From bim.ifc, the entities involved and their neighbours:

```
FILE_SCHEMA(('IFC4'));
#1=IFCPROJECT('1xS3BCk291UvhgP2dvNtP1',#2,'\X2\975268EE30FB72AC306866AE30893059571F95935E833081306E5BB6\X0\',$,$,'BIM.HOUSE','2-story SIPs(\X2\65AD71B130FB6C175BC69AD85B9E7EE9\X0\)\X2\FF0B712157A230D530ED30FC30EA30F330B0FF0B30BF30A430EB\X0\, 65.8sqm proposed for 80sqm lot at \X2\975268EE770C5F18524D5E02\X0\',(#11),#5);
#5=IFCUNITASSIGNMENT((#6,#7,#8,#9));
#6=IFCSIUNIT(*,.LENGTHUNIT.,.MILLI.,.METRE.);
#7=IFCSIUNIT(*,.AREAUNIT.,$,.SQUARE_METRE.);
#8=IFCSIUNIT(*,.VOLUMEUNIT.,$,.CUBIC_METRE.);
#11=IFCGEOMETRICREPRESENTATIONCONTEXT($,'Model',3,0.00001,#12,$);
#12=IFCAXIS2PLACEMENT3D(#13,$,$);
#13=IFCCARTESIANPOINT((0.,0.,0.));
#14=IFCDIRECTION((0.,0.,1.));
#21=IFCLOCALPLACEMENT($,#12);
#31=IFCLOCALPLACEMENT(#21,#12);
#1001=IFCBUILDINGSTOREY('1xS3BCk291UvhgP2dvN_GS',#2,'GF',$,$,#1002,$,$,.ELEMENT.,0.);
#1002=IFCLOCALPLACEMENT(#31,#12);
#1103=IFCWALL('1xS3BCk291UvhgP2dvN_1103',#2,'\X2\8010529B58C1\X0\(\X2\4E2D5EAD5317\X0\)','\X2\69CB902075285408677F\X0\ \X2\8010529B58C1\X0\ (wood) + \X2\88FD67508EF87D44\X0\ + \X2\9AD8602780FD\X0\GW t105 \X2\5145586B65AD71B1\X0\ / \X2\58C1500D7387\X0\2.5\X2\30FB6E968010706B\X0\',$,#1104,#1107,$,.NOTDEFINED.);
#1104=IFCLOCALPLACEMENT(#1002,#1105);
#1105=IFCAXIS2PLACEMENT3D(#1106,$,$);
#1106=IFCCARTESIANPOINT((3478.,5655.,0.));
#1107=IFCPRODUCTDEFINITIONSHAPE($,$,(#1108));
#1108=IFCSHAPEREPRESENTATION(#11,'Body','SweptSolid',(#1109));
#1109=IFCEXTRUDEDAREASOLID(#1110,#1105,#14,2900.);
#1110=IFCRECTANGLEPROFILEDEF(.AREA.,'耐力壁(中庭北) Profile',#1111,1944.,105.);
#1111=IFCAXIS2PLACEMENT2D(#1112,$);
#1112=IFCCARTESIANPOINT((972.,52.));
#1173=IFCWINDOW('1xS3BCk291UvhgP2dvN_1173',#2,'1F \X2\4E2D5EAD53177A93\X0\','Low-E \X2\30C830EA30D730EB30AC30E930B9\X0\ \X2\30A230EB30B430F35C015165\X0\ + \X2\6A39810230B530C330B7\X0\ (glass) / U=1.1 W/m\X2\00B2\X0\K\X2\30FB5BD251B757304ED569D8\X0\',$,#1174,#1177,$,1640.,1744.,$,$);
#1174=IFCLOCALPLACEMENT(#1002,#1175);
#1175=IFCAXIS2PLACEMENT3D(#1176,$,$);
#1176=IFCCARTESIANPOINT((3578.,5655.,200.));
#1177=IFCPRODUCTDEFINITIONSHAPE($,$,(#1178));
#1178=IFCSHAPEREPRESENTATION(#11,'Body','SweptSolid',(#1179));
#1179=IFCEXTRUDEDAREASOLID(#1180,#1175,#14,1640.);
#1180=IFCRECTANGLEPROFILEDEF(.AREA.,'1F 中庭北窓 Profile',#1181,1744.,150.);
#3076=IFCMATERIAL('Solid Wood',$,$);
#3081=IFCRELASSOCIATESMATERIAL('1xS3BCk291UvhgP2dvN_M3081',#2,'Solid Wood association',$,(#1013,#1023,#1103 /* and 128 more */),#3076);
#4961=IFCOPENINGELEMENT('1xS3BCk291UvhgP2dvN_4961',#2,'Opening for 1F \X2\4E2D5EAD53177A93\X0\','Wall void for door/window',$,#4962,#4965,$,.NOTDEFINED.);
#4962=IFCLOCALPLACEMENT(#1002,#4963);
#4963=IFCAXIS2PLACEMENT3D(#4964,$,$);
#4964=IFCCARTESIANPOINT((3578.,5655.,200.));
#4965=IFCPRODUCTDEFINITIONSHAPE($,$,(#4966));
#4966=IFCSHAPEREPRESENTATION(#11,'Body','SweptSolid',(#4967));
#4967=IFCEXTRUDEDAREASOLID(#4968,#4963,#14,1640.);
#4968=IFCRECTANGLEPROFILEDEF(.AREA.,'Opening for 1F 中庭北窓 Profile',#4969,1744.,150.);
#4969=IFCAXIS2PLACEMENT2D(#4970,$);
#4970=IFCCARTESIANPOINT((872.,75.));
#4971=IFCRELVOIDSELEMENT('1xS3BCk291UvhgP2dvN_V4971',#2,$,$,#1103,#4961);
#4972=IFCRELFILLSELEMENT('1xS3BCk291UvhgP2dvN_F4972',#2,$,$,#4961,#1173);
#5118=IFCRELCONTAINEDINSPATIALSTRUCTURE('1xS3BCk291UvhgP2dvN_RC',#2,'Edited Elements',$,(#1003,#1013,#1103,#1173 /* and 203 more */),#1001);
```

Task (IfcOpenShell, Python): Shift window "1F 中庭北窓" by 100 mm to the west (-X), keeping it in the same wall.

```python
import ifcopenshell
import ifcopenshell.api.geometry
import ifcopenshell.util.placement
import ifcopenshell.util.unit

model = ifcopenshell.open("bim.ifc")
unit_scale = ifcopenshell.util.unit.calculate_unit_scale(model)

window = model.by_guid("1xS3BCk291UvhgP2dvN_1173")
opening = window.FillsVoids[0].RelatingOpeningElement
wall = opening.VoidsElements[0].RelatingBuildingElement

wall_matrix = ifcopenshell.util.placement.get_local_placement(wall.ObjectPlacement)
shift = wall_matrix[:3, 0] * -0.1 / unit_scale
before = ifcopenshell.util.placement.get_local_placement(window.ObjectPlacement)[:3, 3].copy()

# The window is not placed relative to its opening, so move both.
for product in (opening, window):
    matrix = ifcopenshell.util.placement.get_local_placement(product.ObjectPlacement)
    matrix[:3, 3] += shift
    ifcopenshell.api.geometry.edit_object_placement(model, product=product, matrix=matrix, is_si=False)

after = ifcopenshell.util.placement.get_local_placement(window.ObjectPlacement)[:3, 3]
print("window moved by", (after - before).round(3) + 0.0)

model.write("bim_rev.ifc")
```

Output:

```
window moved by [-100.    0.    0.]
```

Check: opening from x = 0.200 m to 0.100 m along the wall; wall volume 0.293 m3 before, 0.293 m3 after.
